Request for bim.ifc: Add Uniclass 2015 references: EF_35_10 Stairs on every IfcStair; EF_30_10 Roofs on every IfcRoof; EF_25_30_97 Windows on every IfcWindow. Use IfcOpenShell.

First a look at what the model holds.

```python
import ifcopenshell

model = ifcopenshell.open("bim.ifc")
print(model.schema)
print("classifications:", [c.Name for c in model.by_type("IfcClassification")])
for ifc_class in ("IfcDoor", "IfcRoof", "IfcStair", "IfcWall", "IfcWindow"):
    print(ifc_class, len(model.by_type(ifc_class)))
```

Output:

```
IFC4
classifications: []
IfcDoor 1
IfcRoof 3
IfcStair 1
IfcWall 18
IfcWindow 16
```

```python
import ifcopenshell
import ifcopenshell.api.classification

model = ifcopenshell.open("bim.ifc")

system = ifcopenshell.api.classification.add_classification(model, classification="Uniclass 2015")

codes = {
    "IfcStair": ("EF_35_10", "Stairs"),
    "IfcRoof": ("EF_30_10", "Roofs"),
    "IfcWindow": ("EF_25_30_97", "Windows"),
}
for ifc_class, (code, name) in codes.items():
    products = model.by_type(ifc_class)
    ifcopenshell.api.classification.add_reference(
        model, products=products, classification=system, identification=code, name=name
    )
    print(code, len(products))

model.write("bim_updated.ifc")
```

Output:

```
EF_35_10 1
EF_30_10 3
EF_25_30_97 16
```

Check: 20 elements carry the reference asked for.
